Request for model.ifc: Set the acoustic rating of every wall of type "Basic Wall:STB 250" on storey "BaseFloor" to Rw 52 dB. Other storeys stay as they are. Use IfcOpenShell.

First a look at what the model holds.

```python
import ifcopenshell
import ifcopenshell.util.element

model = ifcopenshell.open("model.ifc")
print(model.schema)
storey = next(s for s in model.by_type("IfcBuildingStorey") if s.Name == "BaseFloor")
walls = [e for e in ifcopenshell.util.element.get_decomposition(storey) if e.is_a("IfcWall")]
seen = {}
for e in walls:
    element_type = ifcopenshell.util.element.get_type(e)
    key = (element_type.Name if element_type != e and element_type else None, ifcopenshell.util.element.get_pset(e, "Pset_WallCommon", "AcousticRating"))
    seen[key] = seen.get(key, 0) + 1
for (name, value), count in sorted(seen.items(), key=str):
    print(count, "x", name, "|", value)
```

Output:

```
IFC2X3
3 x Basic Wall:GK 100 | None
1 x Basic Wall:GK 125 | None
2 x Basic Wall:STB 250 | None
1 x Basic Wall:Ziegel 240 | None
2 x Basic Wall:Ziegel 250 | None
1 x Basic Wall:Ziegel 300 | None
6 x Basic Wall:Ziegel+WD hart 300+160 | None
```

```python
import ifcopenshell
import ifcopenshell.api.pset
import ifcopenshell.util.element

model = ifcopenshell.open("model.ifc")

storey = next(s for s in model.by_type("IfcBuildingStorey") if s.Name == "BaseFloor")
walls = [e for e in ifcopenshell.util.element.get_decomposition(storey) if e.is_a("IfcWall")]

count = 0
for e in walls:
    element_type = ifcopenshell.util.element.get_type(e)
    if element_type in (None, e) or element_type.Name != "Basic Wall:STB 250":
        continue
    # add_pset returns the element's existing set when there is one.
    pset = ifcopenshell.api.pset.add_pset(model, product=e, name="Pset_WallCommon")
    ifcopenshell.api.pset.edit_pset(model, pset=pset, properties={"AcousticRating": "Rw 52 dB"})
    count += 1

print(count, "walls updated")

model.write("model_edited.ifc")
```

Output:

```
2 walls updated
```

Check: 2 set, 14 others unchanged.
